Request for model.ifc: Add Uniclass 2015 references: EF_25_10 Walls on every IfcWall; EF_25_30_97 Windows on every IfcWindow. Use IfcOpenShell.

First a look at what the model holds.

```python
import ifcopenshell

model = ifcopenshell.open("model.ifc")
print(model.schema)
print("classifications:", [c.Name for c in model.by_type("IfcClassification")])
for ifc_class in ("IfcDoor", "IfcRoof", "IfcStair", "IfcWall", "IfcWindow"):
    print(ifc_class, len(model.by_type(ifc_class)))
```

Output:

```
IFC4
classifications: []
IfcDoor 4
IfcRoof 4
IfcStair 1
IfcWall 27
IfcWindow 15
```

```python
import ifcopenshell
import ifcopenshell.api.classification

model = ifcopenshell.open("model.ifc")

system = ifcopenshell.api.classification.add_classification(model, classification="Uniclass 2015")

codes = {
    "IfcWall": ("EF_25_10", "Walls"),
    "IfcWindow": ("EF_25_30_97", "Windows"),
}
for ifc_class, (code, name) in codes.items():
    products = model.by_type(ifc_class)
    ifcopenshell.api.classification.add_reference(
        model, products=products, classification=system, identification=code, name=name
    )
    print(code, len(products))

model.write("model_edited.ifc")
```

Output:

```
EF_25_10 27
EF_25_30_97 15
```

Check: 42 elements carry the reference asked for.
